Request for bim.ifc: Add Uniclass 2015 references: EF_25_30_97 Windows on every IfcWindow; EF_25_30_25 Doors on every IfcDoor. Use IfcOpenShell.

First a look at what the model holds.

```python
import ifcopenshell

model = ifcopenshell.open("bim.ifc")
print(model.schema)
print("classifications:", [c.Name for c in model.by_type("IfcClassification")])
for ifc_class in ("IfcDoor", "IfcRoof", "IfcStair", "IfcWall", "IfcWindow"):
    print(ifc_class, len(model.by_type(ifc_class)))
```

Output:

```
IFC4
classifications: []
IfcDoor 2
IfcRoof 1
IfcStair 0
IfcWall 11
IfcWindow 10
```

```python
import ifcopenshell
import ifcopenshell.api.classification

model = ifcopenshell.open("bim.ifc")

system = ifcopenshell.api.classification.add_classification(model, classification="Uniclass 2015")

codes = {
    "IfcWindow": ("EF_25_30_97", "Windows"),
    "IfcDoor": ("EF_25_30_25", "Doors"),
}
for ifc_class, (code, name) in codes.items():
    products = model.by_type(ifc_class)
    ifcopenshell.api.classification.add_reference(
        model, products=products, classification=system, identification=code, name=name
    )
    print(code, len(products))

model.write("bim_updated.ifc")
```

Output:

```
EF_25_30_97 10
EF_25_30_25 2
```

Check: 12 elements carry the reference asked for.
